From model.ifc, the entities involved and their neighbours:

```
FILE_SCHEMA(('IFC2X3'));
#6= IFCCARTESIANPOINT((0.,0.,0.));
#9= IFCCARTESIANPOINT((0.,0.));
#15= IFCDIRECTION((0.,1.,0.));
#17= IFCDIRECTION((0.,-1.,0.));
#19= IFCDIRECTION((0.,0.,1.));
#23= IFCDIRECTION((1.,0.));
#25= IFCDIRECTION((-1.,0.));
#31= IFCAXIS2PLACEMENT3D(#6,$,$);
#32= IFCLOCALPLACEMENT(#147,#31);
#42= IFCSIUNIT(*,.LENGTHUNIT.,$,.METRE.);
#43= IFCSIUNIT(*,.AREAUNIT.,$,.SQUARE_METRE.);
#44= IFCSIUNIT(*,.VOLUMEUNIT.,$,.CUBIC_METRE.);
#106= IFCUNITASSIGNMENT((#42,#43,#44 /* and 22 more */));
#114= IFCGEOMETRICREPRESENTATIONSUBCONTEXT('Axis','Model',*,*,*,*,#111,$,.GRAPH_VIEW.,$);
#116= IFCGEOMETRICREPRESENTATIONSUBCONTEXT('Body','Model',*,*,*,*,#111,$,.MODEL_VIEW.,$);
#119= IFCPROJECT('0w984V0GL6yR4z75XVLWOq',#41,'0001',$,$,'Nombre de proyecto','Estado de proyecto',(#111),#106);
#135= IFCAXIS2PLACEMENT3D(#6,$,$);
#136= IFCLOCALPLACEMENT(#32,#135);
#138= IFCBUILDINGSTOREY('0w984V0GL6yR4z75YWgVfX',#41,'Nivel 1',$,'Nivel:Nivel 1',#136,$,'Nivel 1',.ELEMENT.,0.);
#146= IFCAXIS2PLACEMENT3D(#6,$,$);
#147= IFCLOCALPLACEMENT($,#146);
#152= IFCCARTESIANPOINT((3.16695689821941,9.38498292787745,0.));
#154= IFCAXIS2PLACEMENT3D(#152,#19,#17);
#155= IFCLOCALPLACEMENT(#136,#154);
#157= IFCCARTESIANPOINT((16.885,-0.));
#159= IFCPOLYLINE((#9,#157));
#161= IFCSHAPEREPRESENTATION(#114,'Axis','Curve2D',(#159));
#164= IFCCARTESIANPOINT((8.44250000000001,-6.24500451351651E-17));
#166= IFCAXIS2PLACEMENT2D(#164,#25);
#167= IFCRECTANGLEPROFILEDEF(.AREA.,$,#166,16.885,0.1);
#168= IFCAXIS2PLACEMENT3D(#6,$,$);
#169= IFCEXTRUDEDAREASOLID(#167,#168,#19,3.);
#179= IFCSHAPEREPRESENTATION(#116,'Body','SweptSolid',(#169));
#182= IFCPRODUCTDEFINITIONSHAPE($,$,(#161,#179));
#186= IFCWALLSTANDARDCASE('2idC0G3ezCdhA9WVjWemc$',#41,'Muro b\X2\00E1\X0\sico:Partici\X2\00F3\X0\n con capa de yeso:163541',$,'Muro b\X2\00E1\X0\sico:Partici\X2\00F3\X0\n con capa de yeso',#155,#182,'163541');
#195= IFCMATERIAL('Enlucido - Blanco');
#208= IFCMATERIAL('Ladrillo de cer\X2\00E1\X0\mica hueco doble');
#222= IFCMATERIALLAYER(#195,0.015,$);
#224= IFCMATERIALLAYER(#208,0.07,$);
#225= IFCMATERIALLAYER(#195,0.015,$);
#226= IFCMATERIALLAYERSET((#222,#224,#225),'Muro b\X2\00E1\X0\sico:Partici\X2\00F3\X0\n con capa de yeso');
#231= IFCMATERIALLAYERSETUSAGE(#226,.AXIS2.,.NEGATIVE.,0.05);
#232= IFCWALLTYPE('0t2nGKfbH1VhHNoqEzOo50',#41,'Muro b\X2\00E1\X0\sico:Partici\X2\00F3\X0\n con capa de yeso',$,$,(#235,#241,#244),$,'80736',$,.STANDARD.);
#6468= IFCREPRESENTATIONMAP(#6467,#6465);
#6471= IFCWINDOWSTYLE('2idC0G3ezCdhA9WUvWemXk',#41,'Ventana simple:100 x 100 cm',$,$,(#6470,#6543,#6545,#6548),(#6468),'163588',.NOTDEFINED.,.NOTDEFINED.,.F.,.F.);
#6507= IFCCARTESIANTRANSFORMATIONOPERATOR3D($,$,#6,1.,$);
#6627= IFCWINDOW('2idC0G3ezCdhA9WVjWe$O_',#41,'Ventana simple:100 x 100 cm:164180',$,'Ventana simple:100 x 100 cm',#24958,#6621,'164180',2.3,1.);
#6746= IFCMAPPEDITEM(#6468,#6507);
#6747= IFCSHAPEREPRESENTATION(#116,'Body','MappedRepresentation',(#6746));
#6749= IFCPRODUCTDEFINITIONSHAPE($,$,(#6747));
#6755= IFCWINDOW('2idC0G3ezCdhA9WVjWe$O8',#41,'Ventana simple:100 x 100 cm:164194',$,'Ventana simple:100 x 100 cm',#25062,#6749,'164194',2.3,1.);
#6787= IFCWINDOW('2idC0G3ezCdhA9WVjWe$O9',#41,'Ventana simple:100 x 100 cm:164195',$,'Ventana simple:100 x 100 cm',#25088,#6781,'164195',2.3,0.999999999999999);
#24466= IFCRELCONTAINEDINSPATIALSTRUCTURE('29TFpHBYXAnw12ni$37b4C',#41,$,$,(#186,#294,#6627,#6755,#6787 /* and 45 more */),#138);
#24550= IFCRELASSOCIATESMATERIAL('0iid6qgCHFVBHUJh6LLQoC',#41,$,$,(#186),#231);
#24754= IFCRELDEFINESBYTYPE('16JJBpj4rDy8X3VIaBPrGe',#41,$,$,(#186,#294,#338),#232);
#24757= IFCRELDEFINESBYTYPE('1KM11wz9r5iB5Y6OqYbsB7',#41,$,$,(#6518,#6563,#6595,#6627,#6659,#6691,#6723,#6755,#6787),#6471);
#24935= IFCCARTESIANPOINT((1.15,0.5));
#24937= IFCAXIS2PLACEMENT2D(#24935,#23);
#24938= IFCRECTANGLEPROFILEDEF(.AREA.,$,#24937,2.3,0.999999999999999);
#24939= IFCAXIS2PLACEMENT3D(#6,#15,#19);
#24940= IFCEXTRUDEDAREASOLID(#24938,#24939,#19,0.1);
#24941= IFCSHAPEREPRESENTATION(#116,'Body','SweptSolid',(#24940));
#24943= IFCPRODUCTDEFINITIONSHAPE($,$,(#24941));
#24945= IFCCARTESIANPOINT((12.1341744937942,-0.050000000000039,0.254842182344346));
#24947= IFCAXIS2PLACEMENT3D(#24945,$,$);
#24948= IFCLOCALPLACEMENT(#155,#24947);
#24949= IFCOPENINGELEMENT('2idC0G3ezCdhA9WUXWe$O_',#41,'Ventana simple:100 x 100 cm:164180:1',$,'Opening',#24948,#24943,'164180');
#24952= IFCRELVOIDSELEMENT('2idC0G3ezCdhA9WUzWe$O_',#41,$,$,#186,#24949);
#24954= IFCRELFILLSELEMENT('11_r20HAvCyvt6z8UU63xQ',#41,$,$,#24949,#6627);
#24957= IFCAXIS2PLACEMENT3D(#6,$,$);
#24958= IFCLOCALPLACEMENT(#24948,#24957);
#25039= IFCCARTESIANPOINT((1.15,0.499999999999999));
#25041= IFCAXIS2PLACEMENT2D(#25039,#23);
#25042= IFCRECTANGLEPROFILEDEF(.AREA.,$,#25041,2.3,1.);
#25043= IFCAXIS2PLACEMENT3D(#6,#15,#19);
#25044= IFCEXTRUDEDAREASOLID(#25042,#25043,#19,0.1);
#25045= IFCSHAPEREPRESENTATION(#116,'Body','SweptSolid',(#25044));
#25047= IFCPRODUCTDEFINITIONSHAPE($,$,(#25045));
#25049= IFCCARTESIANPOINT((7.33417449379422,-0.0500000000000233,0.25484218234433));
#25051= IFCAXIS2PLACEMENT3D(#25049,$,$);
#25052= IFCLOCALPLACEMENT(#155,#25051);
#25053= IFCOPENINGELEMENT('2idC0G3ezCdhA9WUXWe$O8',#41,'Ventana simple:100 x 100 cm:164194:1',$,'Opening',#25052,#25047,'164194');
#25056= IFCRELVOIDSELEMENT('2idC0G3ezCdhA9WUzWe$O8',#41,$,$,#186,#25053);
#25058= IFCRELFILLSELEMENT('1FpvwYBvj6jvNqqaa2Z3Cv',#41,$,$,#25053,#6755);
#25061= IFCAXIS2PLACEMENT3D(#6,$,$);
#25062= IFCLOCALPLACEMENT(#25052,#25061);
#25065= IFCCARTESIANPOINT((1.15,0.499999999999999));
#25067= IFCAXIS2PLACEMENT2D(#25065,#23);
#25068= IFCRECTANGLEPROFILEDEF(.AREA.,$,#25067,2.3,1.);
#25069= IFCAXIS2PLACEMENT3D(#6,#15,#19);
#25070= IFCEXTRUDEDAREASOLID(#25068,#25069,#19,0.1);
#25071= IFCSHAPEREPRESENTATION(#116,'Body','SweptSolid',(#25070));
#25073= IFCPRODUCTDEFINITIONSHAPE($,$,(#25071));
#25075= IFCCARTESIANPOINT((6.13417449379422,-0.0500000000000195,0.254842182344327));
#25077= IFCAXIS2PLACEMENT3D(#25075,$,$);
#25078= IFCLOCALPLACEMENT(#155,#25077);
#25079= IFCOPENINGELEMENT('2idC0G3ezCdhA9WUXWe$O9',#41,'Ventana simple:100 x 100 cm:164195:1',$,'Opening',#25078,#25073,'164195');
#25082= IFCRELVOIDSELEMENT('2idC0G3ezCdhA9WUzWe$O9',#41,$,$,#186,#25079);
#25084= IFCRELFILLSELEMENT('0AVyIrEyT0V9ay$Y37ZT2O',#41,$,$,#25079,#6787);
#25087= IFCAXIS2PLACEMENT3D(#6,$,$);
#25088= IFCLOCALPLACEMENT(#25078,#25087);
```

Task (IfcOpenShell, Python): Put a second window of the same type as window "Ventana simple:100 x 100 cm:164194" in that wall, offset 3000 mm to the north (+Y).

```python
import ifcopenshell
import ifcopenshell.api.feature
import ifcopenshell.api.geometry
import ifcopenshell.api.root
import ifcopenshell.geom
import ifcopenshell.util.element
import ifcopenshell.util.placement
import ifcopenshell.util.shape

model = ifcopenshell.open("model.ifc")
settings = ifcopenshell.geom.settings()


def volume(element):
    """Net volume in cubic metres, openings subtracted."""
    shape = ifcopenshell.geom.create_shape(settings, element)
    return ifcopenshell.util.shape.get_volume(shape.geometry)


def reuse_history(source, copy):
    """copy_class also copies each property set's owner history, people and application; keep the originals."""
    for rel in copy.IsDefinedBy:
        if rel.is_a("IfcRelDefinesByProperties") and (history := rel.RelatingPropertyDefinition.OwnerHistory):
            rel.RelatingPropertyDefinition.OwnerHistory = source.OwnerHistory
            ifcopenshell.util.element.remove_deep2(model, history)


window = model.by_id(6755)
opening = window.FillsVoids[0].RelatingOpeningElement
wall = opening.VoidsElements[0].RelatingBuildingElement
before = volume(wall)
shift = ifcopenshell.util.placement.get_local_placement(wall.ObjectPlacement)[:3, 0] * -3.0

# copy_class copies the void relationship, type, container and properties, but no geometry.
new_opening = ifcopenshell.api.root.copy_class(model, product=opening)
new_opening.Representation = ifcopenshell.util.element.copy_deep(
    model, opening.Representation, exclude=["IfcGeometricRepresentationContext", "IfcRepresentationMap"]
)
new_opening.Name = "Ventana simple:100 x 100 cm"
new_opening.Tag = None
new_window = ifcopenshell.api.root.copy_class(model, product=window)
new_window.Representation = ifcopenshell.util.element.copy_deep(
    model, window.Representation, exclude=["IfcGeometricRepresentationContext", "IfcRepresentationMap"]
)
new_window.Name = "Ventana simple:100 x 100 cm"
new_window.Tag = None
reuse_history(window, new_window)
fills = ifcopenshell.api.feature.add_filling(model, opening=new_opening, element=new_window)
fills.OwnerHistory = new_window.OwnerHistory  # required in IFC2X3

for old, new in ((opening, new_opening), (window, new_window)):
    matrix = ifcopenshell.util.placement.get_local_placement(old.ObjectPlacement)
    matrix[:3, 3] += shift
    ifcopenshell.api.geometry.edit_object_placement(model, product=new, matrix=matrix, is_si=False)

after = volume(wall)

print(f"wall volume {before:.3f} -> {after:.3f} m3")

model.write("model_v2.ifc")
```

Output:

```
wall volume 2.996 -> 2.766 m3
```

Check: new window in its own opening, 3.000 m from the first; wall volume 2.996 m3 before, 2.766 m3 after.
